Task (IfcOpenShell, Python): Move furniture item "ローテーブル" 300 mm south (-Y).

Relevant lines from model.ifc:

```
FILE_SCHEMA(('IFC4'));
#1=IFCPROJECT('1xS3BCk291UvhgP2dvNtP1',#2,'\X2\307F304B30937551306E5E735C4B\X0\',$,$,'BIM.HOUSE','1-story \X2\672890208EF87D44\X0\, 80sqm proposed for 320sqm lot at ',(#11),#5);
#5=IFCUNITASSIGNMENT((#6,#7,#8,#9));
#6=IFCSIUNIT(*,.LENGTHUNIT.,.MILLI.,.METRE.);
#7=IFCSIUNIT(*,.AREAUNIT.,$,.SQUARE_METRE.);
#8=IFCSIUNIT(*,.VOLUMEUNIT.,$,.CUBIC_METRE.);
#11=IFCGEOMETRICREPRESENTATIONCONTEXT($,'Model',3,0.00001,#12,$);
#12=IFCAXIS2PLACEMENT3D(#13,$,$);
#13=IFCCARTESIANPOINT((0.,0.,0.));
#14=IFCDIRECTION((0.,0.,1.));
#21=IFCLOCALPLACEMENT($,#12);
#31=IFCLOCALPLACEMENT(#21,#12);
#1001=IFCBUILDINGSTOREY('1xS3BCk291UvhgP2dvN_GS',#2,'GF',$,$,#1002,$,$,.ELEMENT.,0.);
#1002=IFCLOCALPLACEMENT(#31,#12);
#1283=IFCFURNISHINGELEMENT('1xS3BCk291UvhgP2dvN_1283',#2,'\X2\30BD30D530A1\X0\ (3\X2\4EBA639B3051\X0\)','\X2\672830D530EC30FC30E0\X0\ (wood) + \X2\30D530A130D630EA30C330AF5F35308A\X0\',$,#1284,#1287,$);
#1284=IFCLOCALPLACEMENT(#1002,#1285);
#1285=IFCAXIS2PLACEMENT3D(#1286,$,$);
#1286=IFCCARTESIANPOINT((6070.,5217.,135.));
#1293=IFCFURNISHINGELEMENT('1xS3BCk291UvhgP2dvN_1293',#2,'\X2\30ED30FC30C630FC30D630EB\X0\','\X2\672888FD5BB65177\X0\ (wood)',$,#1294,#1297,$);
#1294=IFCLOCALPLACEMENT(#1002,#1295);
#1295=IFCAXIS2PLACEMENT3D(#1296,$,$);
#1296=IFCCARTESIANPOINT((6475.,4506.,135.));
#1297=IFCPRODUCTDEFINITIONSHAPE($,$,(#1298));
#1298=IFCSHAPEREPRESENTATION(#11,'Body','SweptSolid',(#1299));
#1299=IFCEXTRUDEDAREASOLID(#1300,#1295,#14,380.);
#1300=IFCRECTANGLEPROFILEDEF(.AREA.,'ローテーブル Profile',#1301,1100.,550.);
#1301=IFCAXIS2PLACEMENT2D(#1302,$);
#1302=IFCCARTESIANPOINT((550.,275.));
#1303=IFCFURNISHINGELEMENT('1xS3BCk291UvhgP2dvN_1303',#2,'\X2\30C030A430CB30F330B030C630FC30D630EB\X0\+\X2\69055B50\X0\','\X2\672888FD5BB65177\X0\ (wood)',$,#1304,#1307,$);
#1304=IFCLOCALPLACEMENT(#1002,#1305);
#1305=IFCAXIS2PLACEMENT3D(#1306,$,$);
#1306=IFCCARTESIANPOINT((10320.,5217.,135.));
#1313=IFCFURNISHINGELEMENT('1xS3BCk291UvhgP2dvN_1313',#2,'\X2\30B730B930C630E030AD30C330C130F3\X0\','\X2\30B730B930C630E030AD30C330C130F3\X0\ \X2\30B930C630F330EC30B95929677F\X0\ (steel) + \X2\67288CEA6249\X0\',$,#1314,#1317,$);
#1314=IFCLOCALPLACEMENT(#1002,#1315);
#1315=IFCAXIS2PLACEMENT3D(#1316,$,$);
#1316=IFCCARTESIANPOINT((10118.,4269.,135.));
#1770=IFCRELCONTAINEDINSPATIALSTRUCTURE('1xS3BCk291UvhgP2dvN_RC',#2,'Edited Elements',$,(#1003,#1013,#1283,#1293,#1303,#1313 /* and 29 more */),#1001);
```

```python
import ifcopenshell
import ifcopenshell.api.geometry
import ifcopenshell.util.placement

model = ifcopenshell.open("model.ifc")

item = model.by_guid("1xS3BCk291UvhgP2dvN_1293")
matrix = ifcopenshell.util.placement.get_local_placement(item.ObjectPlacement)
matrix[1, 3] -= 300.0
ifcopenshell.api.geometry.edit_object_placement(model, product=item, matrix=matrix, is_si=False)

print(ifcopenshell.util.placement.get_local_placement(item.ObjectPlacement).round(3) + 0.0)

model.write("model-out.ifc")
```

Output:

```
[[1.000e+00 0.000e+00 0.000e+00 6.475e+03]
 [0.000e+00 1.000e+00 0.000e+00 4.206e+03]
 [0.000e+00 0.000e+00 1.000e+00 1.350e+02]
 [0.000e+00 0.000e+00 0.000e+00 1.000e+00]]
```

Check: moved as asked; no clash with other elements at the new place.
